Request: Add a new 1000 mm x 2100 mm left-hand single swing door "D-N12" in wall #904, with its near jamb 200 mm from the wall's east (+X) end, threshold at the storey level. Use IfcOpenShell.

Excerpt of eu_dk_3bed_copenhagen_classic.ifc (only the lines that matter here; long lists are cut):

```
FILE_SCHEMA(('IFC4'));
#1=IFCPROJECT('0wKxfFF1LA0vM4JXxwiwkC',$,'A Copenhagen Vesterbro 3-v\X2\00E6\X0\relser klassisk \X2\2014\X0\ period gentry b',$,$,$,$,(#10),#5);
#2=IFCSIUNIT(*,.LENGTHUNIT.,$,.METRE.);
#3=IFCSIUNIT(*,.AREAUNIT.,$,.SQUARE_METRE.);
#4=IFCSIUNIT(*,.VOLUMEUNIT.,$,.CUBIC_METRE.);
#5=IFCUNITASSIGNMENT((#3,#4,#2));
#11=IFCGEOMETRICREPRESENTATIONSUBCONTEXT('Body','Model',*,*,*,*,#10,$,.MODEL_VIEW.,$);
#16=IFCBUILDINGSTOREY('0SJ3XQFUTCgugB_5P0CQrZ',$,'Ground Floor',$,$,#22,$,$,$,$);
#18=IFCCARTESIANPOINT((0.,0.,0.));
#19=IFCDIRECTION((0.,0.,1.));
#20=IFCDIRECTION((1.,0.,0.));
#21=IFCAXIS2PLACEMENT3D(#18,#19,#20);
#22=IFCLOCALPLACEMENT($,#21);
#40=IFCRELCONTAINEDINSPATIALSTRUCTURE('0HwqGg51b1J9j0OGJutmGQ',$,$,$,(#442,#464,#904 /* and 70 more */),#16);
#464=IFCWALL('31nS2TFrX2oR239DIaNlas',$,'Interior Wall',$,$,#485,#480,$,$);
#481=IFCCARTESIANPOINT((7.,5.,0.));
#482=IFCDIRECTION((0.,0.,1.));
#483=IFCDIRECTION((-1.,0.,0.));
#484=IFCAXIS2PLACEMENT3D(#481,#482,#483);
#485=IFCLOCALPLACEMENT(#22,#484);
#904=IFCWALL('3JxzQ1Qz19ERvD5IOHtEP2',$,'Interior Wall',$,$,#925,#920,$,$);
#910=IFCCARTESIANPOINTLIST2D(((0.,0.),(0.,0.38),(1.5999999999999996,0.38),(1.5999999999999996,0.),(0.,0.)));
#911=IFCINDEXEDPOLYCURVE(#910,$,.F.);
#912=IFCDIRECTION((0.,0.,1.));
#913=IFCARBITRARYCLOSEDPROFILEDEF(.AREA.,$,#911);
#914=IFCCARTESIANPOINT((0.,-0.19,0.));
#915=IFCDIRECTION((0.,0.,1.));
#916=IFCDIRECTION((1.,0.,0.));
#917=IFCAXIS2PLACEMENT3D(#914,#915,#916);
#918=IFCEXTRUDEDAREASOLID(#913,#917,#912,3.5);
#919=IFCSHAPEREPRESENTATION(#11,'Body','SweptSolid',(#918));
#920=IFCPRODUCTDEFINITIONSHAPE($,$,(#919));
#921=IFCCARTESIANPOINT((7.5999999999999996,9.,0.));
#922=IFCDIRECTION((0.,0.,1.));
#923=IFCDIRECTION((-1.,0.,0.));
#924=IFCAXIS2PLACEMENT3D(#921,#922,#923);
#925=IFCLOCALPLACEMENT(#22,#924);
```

```python
import numpy as np
import ifcopenshell
import ifcopenshell.api.feature
import ifcopenshell.api.geometry
import ifcopenshell.api.root
import ifcopenshell.api.spatial
import ifcopenshell.geom
import ifcopenshell.util.element
import ifcopenshell.util.placement
import ifcopenshell.util.representation
import ifcopenshell.util.shape
import ifcopenshell.util.unit

model = ifcopenshell.open("eu_dk_3bed_copenhagen_classic.ifc")
unit_scale = ifcopenshell.util.unit.calculate_unit_scale(model)
settings = ifcopenshell.geom.settings()


def volume(element):
    """Net volume in cubic metres, openings subtracted."""
    shape = ifcopenshell.geom.create_shape(settings, element)
    return ifcopenshell.util.shape.get_volume(shape.geometry)


wall = model.by_guid("3JxzQ1Qz19ERvD5IOHtEP2")
storey = ifcopenshell.util.element.get_container(wall, ifc_class="IfcBuildingStorey")
context = ifcopenshell.util.representation.get_context(model, "Model", "Body", "MODEL_VIEW")
before = volume(wall)

width, height, from_end, sill = 1, 2.1, 0.2, 0.0  # metres

# The wall runs along its own X axis, and the end named is its -X end.
wall_shape = ifcopenshell.geom.create_shape(settings, wall)
x, y, z = ifcopenshell.util.shape.get_vertices(wall_shape.geometry).T
start = x.min() + from_end
face, thickness = float(y.min()), float(y.max() - y.min())
wall_matrix = ifcopenshell.util.placement.get_local_placement(wall.ObjectPlacement)
level = ifcopenshell.util.placement.get_local_placement(storey.ObjectPlacement)[2, 3]


def in_wall(x, y):
    """Placement at x, y metres in the wall's axes, at sill height."""
    matrix = wall_matrix.copy()
    matrix[:, 3] = wall_matrix @ np.array([x / unit_scale, y / unit_scale, 0.0, 1.0])
    matrix[2, 3] = level + sill / unit_scale
    return matrix


# Opening: a box that overshoots both wall faces by 50 mm.
opening = ifcopenshell.api.root.create_entity(model, ifc_class="IfcOpeningElement", predefined_type="OPENING")
box = ifcopenshell.api.geometry.add_wall_representation(
    model, context=context, length=width, height=height, thickness=thickness + 0.1
)
ifcopenshell.api.geometry.assign_representation(model, product=opening, representation=box)
ifcopenshell.api.geometry.edit_object_placement(model, product=opening, matrix=in_wall(start, face - 0.05), is_si=False)
ifcopenshell.api.feature.add_feature(model, feature=opening, element=wall)

door = ifcopenshell.api.root.create_entity(model, ifc_class="IfcDoor", name="D-N12", predefined_type="DOOR")
door.OverallWidth, door.OverallHeight = width / unit_scale, height / unit_scale
door.OperationType = "SINGLE_SWING_LEFT"
body = ifcopenshell.api.geometry.add_door_representation(
    model,
    context=context,
    overall_width=door.OverallWidth,
    overall_height=door.OverallHeight,
    operation_type="SINGLE_SWING_LEFT",
    lining_properties={"LiningDepth": thickness / unit_scale, "ThresholdDepth": thickness / unit_scale},
)
ifcopenshell.api.geometry.assign_representation(model, product=door, representation=body)
ifcopenshell.api.spatial.assign_container(model, products=[door], relating_structure=storey)
ifcopenshell.api.feature.add_filling(model, opening=opening, element=door)

# The lining spans the wall, so the door starts at the wall face.
ifcopenshell.api.geometry.edit_object_placement(model, product=door, matrix=in_wall(start, face), is_si=False)

after = volume(wall)

print(f"wall volume {before:.3f} -> {after:.3f} m3")

model.write("eu_dk_3bed_copenhagen_classic_rev.ifc")
```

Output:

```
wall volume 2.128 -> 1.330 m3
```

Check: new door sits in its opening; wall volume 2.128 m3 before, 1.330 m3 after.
